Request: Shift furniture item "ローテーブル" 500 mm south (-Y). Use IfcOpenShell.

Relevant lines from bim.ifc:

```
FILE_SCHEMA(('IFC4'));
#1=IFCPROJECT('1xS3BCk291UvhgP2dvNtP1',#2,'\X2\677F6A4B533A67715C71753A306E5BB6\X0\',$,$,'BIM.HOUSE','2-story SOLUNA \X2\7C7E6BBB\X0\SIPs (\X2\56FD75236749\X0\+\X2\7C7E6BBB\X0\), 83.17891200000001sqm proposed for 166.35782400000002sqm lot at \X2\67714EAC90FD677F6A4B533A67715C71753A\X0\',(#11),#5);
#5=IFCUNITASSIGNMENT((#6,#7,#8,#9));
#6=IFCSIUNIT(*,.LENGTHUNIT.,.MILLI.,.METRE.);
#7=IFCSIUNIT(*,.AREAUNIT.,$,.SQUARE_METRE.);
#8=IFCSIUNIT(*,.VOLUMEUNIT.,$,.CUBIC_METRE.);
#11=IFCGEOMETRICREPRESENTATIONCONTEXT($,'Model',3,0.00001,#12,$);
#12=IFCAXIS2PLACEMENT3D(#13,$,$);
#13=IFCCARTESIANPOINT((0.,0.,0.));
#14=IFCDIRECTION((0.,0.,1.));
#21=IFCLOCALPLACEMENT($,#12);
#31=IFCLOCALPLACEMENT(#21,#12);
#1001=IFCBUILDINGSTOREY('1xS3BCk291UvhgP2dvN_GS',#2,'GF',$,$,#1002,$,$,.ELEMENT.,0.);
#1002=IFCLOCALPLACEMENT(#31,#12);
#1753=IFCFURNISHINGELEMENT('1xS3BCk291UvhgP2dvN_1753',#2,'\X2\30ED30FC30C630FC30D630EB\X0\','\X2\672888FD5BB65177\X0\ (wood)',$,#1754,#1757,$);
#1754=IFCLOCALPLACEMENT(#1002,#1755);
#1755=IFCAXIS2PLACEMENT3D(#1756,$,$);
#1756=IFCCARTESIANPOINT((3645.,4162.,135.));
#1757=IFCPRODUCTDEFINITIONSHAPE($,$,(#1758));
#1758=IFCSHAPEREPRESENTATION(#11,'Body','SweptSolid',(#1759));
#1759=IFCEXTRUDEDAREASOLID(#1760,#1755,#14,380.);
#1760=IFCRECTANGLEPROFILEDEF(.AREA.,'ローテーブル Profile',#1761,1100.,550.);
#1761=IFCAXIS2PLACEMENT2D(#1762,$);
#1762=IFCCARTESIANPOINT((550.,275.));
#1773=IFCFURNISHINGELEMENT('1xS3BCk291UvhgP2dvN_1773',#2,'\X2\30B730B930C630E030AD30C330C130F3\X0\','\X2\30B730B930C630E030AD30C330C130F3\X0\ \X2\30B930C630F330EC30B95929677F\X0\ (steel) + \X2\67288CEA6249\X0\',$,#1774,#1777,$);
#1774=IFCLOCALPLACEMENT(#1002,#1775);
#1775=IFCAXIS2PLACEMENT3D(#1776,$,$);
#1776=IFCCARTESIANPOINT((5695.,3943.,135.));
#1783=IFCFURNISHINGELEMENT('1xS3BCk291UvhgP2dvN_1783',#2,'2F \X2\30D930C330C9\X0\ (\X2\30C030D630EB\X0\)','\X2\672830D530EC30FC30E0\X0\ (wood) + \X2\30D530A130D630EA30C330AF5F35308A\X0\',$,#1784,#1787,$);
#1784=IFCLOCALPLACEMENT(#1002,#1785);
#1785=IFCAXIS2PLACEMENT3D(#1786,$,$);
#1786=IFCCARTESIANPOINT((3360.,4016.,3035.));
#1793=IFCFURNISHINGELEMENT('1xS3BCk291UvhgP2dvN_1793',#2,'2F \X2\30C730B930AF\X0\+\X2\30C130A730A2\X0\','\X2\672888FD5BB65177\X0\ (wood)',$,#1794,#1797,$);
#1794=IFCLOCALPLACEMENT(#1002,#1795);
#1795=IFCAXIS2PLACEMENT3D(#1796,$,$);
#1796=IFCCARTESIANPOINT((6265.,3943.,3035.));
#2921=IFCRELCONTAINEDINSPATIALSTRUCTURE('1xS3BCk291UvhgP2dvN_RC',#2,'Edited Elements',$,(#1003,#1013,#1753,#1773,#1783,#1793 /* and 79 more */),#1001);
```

```python
import ifcopenshell
import ifcopenshell.api.geometry
import ifcopenshell.util.placement

model = ifcopenshell.open("bim.ifc")

item = model.by_id(1753)
matrix = ifcopenshell.util.placement.get_local_placement(item.ObjectPlacement)
matrix[1, 3] -= 500.0
ifcopenshell.api.geometry.edit_object_placement(model, product=item, matrix=matrix, is_si=False)

print(ifcopenshell.util.placement.get_local_placement(item.ObjectPlacement).round(3) + 0.0)

model.write("bim_updated.ifc")
```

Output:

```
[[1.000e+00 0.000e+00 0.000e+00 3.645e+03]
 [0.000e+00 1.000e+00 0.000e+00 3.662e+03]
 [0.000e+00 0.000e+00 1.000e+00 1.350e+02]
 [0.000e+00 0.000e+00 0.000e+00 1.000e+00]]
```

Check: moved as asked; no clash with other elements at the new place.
